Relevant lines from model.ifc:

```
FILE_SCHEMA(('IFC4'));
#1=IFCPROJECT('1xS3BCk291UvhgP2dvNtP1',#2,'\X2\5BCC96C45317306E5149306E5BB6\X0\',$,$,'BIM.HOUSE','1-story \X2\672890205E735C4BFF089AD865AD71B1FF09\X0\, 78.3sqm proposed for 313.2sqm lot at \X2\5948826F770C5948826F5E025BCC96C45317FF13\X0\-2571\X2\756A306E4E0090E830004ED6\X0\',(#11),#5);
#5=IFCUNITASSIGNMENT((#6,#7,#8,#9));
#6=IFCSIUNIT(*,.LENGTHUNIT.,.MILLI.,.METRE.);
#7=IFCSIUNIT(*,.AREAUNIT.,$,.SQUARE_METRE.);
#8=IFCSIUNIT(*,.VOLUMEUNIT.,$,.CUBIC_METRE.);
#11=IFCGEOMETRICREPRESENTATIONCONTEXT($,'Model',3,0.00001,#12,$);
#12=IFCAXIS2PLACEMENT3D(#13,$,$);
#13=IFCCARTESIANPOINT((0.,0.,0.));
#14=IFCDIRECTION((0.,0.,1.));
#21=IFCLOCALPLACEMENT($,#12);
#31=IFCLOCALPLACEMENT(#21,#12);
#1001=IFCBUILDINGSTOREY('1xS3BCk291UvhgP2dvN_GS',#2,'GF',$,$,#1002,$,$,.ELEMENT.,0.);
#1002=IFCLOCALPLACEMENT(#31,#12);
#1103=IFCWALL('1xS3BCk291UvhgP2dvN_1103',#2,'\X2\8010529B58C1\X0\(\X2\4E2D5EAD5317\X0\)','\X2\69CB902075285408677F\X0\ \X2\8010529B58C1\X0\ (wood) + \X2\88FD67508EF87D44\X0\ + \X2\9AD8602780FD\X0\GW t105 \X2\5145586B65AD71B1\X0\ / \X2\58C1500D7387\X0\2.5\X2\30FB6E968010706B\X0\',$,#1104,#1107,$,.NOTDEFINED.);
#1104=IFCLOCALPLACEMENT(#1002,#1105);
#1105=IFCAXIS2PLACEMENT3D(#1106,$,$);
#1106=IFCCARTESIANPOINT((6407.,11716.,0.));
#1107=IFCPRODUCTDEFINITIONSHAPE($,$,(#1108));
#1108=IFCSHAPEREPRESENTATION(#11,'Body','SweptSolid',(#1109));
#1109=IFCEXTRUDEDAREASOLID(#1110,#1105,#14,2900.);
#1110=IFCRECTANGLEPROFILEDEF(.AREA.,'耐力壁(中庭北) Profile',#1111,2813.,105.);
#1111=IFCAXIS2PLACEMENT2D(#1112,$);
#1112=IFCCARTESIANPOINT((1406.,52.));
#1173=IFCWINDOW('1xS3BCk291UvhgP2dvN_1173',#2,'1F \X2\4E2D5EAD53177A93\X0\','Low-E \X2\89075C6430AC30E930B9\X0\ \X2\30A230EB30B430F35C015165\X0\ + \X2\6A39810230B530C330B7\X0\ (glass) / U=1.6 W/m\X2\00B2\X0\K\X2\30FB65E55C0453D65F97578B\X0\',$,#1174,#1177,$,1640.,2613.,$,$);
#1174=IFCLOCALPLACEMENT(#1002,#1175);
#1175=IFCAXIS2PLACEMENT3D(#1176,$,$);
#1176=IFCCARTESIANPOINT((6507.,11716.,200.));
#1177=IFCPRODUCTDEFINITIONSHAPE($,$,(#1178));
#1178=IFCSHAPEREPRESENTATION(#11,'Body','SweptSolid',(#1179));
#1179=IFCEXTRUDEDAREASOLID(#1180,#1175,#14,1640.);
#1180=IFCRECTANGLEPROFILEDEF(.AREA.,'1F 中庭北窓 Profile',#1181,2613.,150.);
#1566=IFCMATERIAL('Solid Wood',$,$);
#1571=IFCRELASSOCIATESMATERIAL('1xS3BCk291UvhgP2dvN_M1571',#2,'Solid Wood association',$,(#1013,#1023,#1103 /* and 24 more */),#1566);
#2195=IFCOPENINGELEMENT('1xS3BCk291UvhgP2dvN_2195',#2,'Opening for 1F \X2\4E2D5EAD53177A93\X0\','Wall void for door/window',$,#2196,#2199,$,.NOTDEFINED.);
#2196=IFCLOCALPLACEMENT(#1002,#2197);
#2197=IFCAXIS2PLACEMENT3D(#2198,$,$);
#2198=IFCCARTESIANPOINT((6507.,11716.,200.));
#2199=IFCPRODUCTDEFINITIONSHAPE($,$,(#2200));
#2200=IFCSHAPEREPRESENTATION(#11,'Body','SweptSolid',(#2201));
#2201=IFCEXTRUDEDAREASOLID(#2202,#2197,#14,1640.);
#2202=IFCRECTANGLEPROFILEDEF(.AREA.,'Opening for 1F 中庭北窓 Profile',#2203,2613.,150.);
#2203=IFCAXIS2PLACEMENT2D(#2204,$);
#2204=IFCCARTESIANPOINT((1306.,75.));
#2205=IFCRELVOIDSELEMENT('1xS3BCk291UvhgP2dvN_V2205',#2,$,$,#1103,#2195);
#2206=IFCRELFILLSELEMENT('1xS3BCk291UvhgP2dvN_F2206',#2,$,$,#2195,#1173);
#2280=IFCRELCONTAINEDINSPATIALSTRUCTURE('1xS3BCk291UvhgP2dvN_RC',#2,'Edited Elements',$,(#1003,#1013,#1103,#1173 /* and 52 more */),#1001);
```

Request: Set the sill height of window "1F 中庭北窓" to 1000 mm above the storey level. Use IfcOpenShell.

```python
import numpy as np
import ifcopenshell
import ifcopenshell.api.geometry
import ifcopenshell.geom
import ifcopenshell.util.element
import ifcopenshell.util.placement
import ifcopenshell.util.shape
import ifcopenshell.util.unit

model = ifcopenshell.open("model.ifc")
unit_scale = ifcopenshell.util.unit.calculate_unit_scale(model)

window = model.by_guid("1xS3BCk291UvhgP2dvN_1173")
opening = window.FillsVoids[0].RelatingOpeningElement
storey = ifcopenshell.util.element.get_container(window, ifc_class="IfcBuildingStorey")
level = ifcopenshell.util.placement.get_local_placement(storey.ObjectPlacement)[2, 3]

# The opening's origin need not be at the sill, so measure its lowest point.
shape = ifcopenshell.geom.create_shape(ifcopenshell.geom.settings(), opening)
bottom = ifcopenshell.util.shape.get_shape_bottom_elevation(shape, shape.geometry) / unit_scale
dz = level + 1 / unit_scale - bottom

shift = np.array([0.0, 0.0, dz])
# The window is not placed relative to its opening, so move both.
for product in (opening, window):
    matrix = ifcopenshell.util.placement.get_local_placement(product.ObjectPlacement)
    matrix[:3, 3] += shift
    ifcopenshell.api.geometry.edit_object_placement(model, product=product, matrix=matrix, is_si=False)

print(f"moved by {dz * unit_scale:+.3f} m")

model.write("model_updated.ifc")
```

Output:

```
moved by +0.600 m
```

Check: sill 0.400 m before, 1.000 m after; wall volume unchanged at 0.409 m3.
